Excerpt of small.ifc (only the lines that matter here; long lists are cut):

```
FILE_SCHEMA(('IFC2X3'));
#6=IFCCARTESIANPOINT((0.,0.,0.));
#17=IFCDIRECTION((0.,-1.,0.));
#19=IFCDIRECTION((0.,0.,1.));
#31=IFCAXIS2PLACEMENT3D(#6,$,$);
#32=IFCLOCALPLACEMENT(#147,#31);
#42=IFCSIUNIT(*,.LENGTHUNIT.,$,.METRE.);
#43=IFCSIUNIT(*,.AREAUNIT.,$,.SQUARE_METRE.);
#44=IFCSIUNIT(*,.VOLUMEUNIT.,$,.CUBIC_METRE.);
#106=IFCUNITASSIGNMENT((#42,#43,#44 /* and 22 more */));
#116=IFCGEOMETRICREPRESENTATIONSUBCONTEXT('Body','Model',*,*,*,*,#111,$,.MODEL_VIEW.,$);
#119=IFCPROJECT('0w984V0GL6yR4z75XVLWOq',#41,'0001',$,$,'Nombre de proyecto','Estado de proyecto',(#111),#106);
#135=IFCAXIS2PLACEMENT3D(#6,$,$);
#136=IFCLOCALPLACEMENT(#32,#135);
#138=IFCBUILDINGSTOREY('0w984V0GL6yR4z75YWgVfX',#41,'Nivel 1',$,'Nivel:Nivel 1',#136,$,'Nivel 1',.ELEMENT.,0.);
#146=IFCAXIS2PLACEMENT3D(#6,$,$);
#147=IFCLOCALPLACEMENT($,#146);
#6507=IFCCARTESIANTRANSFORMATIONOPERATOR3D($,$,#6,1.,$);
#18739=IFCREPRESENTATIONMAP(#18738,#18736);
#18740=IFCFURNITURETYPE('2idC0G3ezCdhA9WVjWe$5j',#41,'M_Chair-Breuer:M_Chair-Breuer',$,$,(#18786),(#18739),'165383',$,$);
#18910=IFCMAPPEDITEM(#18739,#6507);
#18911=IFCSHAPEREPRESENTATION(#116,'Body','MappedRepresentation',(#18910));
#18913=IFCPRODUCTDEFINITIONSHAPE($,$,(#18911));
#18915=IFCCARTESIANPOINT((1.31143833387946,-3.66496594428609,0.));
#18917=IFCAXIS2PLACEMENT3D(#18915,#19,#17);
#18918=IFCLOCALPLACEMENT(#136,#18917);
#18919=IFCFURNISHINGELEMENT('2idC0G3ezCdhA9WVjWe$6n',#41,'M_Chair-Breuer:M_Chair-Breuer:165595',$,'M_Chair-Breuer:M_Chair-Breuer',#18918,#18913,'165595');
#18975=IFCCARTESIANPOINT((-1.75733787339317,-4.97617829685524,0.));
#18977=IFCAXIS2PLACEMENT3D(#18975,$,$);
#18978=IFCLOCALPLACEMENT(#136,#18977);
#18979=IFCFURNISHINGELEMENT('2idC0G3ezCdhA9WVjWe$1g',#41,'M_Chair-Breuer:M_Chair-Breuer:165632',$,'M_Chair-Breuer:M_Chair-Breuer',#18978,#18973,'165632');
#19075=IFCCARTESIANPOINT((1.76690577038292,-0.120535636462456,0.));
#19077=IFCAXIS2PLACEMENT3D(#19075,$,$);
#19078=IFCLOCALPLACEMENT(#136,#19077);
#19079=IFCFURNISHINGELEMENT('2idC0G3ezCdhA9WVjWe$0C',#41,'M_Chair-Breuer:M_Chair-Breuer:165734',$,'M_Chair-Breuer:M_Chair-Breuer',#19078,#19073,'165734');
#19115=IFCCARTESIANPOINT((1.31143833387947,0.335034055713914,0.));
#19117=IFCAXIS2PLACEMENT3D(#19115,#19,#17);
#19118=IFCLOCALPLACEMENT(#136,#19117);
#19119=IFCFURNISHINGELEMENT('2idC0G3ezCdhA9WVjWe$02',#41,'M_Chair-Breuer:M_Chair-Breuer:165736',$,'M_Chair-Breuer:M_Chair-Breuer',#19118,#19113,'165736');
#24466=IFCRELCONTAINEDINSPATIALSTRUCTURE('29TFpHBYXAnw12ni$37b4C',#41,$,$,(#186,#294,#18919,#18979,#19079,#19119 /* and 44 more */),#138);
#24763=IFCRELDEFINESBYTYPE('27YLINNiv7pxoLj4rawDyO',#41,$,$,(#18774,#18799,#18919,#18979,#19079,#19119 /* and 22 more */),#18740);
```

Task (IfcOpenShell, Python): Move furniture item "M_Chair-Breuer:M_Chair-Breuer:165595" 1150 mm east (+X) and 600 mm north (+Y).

```python
import ifcopenshell
import ifcopenshell.api.geometry
import ifcopenshell.util.placement

model = ifcopenshell.open("small.ifc")

item = model.by_guid("2idC0G3ezCdhA9WVjWe$6n")
matrix = ifcopenshell.util.placement.get_local_placement(item.ObjectPlacement)
matrix[0, 3] += 1.15
matrix[1, 3] += 0.6
ifcopenshell.api.geometry.edit_object_placement(model, product=item, matrix=matrix, is_si=False)

print(ifcopenshell.util.placement.get_local_placement(item.ObjectPlacement).round(3) + 0.0)

model.write("small_v2.ifc")
```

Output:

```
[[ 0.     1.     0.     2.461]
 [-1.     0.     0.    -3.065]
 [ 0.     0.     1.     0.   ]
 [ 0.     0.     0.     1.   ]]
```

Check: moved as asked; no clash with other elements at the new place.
